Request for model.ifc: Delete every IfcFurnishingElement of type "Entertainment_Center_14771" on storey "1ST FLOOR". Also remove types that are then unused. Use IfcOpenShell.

First a look at what the model holds.

```python
import ifcopenshell
import ifcopenshell.util.element

model = ifcopenshell.open("model.ifc")
print(model.schema)
storey = next(s for s in model.by_type("IfcBuildingStorey") if s.Name == "1ST FLOOR")
furniture = [e for e in ifcopenshell.util.element.get_decomposition(storey) if e.is_a("IfcFurnishingElement")]
seen = {}
for e in furniture:
    element_type = ifcopenshell.util.element.get_type(e)
    name = element_type.Name if element_type not in (None, e) else None
    seen[name] = seen.get(name, 0) + 1
for name, count in sorted(seen.items(), key=str):
    print(count, "x", name)
```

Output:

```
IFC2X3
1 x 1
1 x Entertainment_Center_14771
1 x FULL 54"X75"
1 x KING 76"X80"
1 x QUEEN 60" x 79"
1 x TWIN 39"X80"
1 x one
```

```python
import ifcopenshell
import ifcopenshell.api.root
import ifcopenshell.util.element

model = ifcopenshell.open("model.ifc")

storey = next(s for s in model.by_type("IfcBuildingStorey") if s.Name == "1ST FLOOR")
furniture = [e for e in ifcopenshell.util.element.get_decomposition(storey) if e.is_a("IfcFurnishingElement")]
targets = [e for e in furniture if (t := ifcopenshell.util.element.get_type(e)) not in (None, e) and t.Name == "Entertainment_Center_14771"]
types = {ifcopenshell.util.element.get_type(e) for e in targets} - {None, *targets}

for e in targets:
    ifcopenshell.api.root.remove_product(model, product=e)
print(len(targets), "removed")

unused = [t for t in types if not ifcopenshell.util.element.get_types(t)]
for t in unused:
    ifcopenshell.api.root.remove_product(model, product=t)
print(len(unused), "unused types removed")

model.write("model_v2.ifc")
```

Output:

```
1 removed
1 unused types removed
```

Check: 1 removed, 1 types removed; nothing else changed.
